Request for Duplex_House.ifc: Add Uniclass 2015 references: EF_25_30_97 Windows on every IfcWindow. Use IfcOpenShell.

First a look at what the model holds.

```python
import ifcopenshell

model = ifcopenshell.open("Duplex_House.ifc")
print(model.schema)
print("classifications:", [c.Name for c in model.by_type("IfcClassification")])
for ifc_class in ("IfcDoor", "IfcRoof", "IfcStair", "IfcWall", "IfcWindow"):
    print(ifc_class, len(model.by_type(ifc_class)))
```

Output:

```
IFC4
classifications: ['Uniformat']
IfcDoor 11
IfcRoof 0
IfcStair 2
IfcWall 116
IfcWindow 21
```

```python
import ifcopenshell
import ifcopenshell.api.classification

model = ifcopenshell.open("Duplex_House.ifc")

system = ifcopenshell.api.classification.add_classification(model, classification="Uniclass 2015")

codes = {
    "IfcWindow": ("EF_25_30_97", "Windows"),
}
for ifc_class, (code, name) in codes.items():
    products = model.by_type(ifc_class)
    ifcopenshell.api.classification.add_reference(
        model, products=products, classification=system, identification=code, name=name
    )
    print(code, len(products))

model.write("Duplex_House_v2.ifc")
```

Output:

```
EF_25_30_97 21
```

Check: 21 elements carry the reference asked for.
